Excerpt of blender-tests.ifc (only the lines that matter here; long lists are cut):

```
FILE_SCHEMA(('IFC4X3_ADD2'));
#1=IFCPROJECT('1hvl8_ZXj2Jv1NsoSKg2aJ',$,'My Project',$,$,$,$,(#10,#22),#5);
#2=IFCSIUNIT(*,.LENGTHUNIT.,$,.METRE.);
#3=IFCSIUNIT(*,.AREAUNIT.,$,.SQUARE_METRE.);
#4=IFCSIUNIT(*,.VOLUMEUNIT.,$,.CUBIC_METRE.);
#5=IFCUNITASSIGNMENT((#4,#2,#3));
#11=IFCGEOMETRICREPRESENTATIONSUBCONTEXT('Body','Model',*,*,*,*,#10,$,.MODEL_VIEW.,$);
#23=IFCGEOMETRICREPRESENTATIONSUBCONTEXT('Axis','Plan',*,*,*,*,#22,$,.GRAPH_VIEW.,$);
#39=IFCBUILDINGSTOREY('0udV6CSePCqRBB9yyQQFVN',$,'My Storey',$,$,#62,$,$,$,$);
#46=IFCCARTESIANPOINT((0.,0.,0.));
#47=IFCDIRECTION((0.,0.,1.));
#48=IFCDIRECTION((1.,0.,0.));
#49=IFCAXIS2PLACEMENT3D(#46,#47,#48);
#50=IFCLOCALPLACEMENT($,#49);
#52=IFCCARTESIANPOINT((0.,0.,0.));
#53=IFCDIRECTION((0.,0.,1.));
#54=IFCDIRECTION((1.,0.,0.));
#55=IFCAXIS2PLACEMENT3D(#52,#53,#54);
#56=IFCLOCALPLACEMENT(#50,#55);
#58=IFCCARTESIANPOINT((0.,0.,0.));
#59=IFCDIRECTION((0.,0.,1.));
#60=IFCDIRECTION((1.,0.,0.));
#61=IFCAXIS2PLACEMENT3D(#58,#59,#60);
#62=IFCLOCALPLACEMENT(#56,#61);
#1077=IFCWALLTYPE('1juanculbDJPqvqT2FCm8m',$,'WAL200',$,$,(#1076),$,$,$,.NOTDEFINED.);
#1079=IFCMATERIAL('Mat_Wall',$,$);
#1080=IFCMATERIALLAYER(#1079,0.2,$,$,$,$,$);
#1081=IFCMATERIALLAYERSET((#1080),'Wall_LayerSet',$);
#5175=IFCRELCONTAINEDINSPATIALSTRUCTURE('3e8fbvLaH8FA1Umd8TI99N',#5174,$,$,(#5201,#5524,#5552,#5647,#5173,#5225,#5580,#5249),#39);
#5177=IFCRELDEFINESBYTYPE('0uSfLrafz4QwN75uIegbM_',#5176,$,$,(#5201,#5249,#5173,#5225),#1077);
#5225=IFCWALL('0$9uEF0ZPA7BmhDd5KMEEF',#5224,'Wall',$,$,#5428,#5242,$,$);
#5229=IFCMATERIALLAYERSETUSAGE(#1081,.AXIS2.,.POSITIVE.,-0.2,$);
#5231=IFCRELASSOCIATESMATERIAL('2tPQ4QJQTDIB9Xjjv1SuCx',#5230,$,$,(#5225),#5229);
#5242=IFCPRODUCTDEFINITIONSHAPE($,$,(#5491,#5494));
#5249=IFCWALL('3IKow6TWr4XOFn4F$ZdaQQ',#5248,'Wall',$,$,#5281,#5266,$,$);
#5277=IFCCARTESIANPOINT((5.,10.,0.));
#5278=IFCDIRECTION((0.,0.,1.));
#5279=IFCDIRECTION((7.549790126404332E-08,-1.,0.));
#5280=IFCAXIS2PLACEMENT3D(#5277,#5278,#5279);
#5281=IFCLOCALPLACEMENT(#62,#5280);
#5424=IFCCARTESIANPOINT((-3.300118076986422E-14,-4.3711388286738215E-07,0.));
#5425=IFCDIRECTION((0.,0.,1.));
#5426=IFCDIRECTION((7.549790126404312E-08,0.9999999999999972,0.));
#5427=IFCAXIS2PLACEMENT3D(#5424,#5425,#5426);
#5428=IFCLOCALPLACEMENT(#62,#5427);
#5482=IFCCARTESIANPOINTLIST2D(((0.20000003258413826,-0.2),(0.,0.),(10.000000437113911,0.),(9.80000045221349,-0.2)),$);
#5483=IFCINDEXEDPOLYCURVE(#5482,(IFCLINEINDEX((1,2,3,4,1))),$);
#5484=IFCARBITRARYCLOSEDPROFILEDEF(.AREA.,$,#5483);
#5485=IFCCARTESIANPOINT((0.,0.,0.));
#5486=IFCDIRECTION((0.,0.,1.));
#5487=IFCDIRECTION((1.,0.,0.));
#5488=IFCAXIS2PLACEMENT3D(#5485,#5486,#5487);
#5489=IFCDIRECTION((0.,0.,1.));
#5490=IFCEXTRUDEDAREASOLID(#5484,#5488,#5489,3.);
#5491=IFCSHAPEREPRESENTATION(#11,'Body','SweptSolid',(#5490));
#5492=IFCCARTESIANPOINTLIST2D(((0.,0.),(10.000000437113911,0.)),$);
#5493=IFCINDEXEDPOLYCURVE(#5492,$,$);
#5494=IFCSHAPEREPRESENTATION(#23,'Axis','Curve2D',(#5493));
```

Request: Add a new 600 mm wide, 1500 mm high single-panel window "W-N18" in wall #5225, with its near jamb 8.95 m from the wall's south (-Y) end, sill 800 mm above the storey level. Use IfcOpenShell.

```python
import numpy as np
import ifcopenshell
import ifcopenshell.api.feature
import ifcopenshell.api.geometry
import ifcopenshell.api.root
import ifcopenshell.api.spatial
import ifcopenshell.geom
import ifcopenshell.util.element
import ifcopenshell.util.placement
import ifcopenshell.util.representation
import ifcopenshell.util.shape
import ifcopenshell.util.unit

model = ifcopenshell.open("blender-tests.ifc")
unit_scale = ifcopenshell.util.unit.calculate_unit_scale(model)
settings = ifcopenshell.geom.settings()


def volume(element):
    """Net volume in cubic metres, openings subtracted."""
    shape = ifcopenshell.geom.create_shape(settings, element)
    return ifcopenshell.util.shape.get_volume(shape.geometry)


wall = model.by_guid("0$9uEF0ZPA7BmhDd5KMEEF")
storey = ifcopenshell.util.element.get_container(wall, ifc_class="IfcBuildingStorey")
context = ifcopenshell.util.representation.get_context(model, "Model", "Body", "MODEL_VIEW")
before = volume(wall)

width, height, from_end, sill = 0.6, 1.5, 8.95, 0.8  # metres

# The wall runs along its own X axis, and the end named is its -X end.
wall_shape = ifcopenshell.geom.create_shape(settings, wall)
x, y, z = ifcopenshell.util.shape.get_vertices(wall_shape.geometry).T
start = x.min() + from_end
face, thickness = float(y.min()), float(y.max() - y.min())
wall_matrix = ifcopenshell.util.placement.get_local_placement(wall.ObjectPlacement)
level = ifcopenshell.util.placement.get_local_placement(storey.ObjectPlacement)[2, 3]


def in_wall(x, y):
    """Placement at x, y metres in the wall's axes, at sill height."""
    matrix = wall_matrix.copy()
    matrix[:, 3] = wall_matrix @ np.array([x / unit_scale, y / unit_scale, 0.0, 1.0])
    matrix[2, 3] = level + sill / unit_scale
    return matrix


# Opening: a box that overshoots both wall faces by 50 mm.
opening = ifcopenshell.api.root.create_entity(model, ifc_class="IfcOpeningElement", predefined_type="OPENING")
box = ifcopenshell.api.geometry.add_wall_representation(
    model, context=context, length=width, height=height, thickness=thickness + 0.1
)
ifcopenshell.api.geometry.assign_representation(model, product=opening, representation=box)
ifcopenshell.api.geometry.edit_object_placement(model, product=opening, matrix=in_wall(start, face - 0.05), is_si=False)
ifcopenshell.api.feature.add_feature(model, feature=opening, element=wall)

window = ifcopenshell.api.root.create_entity(model, ifc_class="IfcWindow", name="W-N18", predefined_type="WINDOW")
window.OverallWidth, window.OverallHeight = width / unit_scale, height / unit_scale
window.PartitioningType = "SINGLE_PANEL"
body = ifcopenshell.api.geometry.add_window_representation(
    model,
    context=context,
    overall_width=window.OverallWidth,
    overall_height=window.OverallHeight,
    partition_type="SINGLE_PANEL",
)
ifcopenshell.api.geometry.assign_representation(model, product=window, representation=body)
ifcopenshell.api.spatial.assign_container(model, products=[window], relating_structure=storey)
ifcopenshell.api.feature.add_filling(model, opening=opening, element=window)

# Centre the window in the wall's thickness.
ifcopenshell.api.geometry.edit_object_placement(model, product=window, matrix=in_wall(start, face), is_si=False)
window_shape = ifcopenshell.geom.create_shape(settings, window)
depth = ifcopenshell.util.shape.get_vertices(window_shape.geometry)[:, 1]
offset = face + thickness / 2 - (depth.min() + depth.max()) / 2
ifcopenshell.api.geometry.edit_object_placement(model, product=window, matrix=in_wall(start, offset), is_si=False)

after = volume(wall)

print(f"wall volume {before:.3f} -> {after:.3f} m3")

model.write("blender-tests_v2.ifc")
```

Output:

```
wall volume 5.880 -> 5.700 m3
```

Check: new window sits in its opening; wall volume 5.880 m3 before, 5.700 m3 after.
